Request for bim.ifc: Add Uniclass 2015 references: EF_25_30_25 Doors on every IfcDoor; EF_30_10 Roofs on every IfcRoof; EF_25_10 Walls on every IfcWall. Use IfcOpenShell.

First a look at what the model holds.

```python
import ifcopenshell

model = ifcopenshell.open("bim.ifc")
print(model.schema)
print("classifications:", [c.Name for c in model.by_type("IfcClassification")])
for ifc_class in ("IfcDoor", "IfcRoof", "IfcStair", "IfcWall", "IfcWindow"):
    print(ifc_class, len(model.by_type(ifc_class)))
```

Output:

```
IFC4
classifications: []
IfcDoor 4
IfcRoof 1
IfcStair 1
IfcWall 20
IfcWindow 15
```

```python
import ifcopenshell
import ifcopenshell.api.classification

model = ifcopenshell.open("bim.ifc")

system = ifcopenshell.api.classification.add_classification(model, classification="Uniclass 2015")

codes = {
    "IfcDoor": ("EF_25_30_25", "Doors"),
    "IfcRoof": ("EF_30_10", "Roofs"),
    "IfcWall": ("EF_25_10", "Walls"),
}
for ifc_class, (code, name) in codes.items():
    products = model.by_type(ifc_class)
    ifcopenshell.api.classification.add_reference(
        model, products=products, classification=system, identification=code, name=name
    )
    print(code, len(products))

model.write("bim-out.ifc")
```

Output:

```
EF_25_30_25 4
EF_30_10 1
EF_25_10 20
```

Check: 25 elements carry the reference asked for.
